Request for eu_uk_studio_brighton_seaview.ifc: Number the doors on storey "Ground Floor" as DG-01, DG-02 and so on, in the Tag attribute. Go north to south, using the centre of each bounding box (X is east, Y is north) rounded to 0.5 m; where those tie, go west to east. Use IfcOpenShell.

First a look at what the model holds.

```python
import ifcopenshell
import ifcopenshell.util.element
import ifcopenshell.util.placement

model = ifcopenshell.open("eu_uk_studio_brighton_seaview.ifc")
print(model.schema)
storey = next(s for s in model.by_type("IfcBuildingStorey") if s.Name == "Ground Floor")
doors = [e for e in ifcopenshell.util.element.get_decomposition(storey) if e.is_a("IfcDoor")]
for e in sorted(doors, key=lambda e: e.id()):
    origin = ifcopenshell.util.placement.get_local_placement(e.ObjectPlacement)[:3, 3]
    print(e.id(), e.Tag, e.Name, origin.round(2) + 0.0, sep=" | ")
```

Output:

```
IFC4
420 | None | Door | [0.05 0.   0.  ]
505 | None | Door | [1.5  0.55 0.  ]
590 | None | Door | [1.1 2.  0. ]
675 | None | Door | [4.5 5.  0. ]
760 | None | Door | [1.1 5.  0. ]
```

```python
import ifcopenshell
import ifcopenshell.geom
import ifcopenshell.util.element
import ifcopenshell.util.shape

model = ifcopenshell.open("eu_uk_studio_brighton_seaview.ifc")
settings = ifcopenshell.geom.settings()
settings.set("use-world-coords", True)


def centre(element):
    shape = ifcopenshell.geom.create_shape(settings, element)
    return ifcopenshell.util.shape.get_bbox_centroid(shape.geometry)


storey = next(s for s in model.by_type("IfcBuildingStorey") if s.Name == "Ground Floor")
doors = [e for e in ifcopenshell.util.element.get_decomposition(storey) if e.is_a("IfcDoor")]

# Insertion points can sit at a corner or the storey origin, so sort by the geometry (in metres).
centres = {e: centre(e) for e in doors}
doors.sort(key=lambda e: (-round(centres[e][1] / 0.5), centres[e][0]))

for i, e in enumerate(doors, start=1):
    number = f"DG-{i:02d}"
    e.Tag = number
    print(e.id(), number)

model.write("eu_uk_studio_brighton_seaview-out.ifc")
```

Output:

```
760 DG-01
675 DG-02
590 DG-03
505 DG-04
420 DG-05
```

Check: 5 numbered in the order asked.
